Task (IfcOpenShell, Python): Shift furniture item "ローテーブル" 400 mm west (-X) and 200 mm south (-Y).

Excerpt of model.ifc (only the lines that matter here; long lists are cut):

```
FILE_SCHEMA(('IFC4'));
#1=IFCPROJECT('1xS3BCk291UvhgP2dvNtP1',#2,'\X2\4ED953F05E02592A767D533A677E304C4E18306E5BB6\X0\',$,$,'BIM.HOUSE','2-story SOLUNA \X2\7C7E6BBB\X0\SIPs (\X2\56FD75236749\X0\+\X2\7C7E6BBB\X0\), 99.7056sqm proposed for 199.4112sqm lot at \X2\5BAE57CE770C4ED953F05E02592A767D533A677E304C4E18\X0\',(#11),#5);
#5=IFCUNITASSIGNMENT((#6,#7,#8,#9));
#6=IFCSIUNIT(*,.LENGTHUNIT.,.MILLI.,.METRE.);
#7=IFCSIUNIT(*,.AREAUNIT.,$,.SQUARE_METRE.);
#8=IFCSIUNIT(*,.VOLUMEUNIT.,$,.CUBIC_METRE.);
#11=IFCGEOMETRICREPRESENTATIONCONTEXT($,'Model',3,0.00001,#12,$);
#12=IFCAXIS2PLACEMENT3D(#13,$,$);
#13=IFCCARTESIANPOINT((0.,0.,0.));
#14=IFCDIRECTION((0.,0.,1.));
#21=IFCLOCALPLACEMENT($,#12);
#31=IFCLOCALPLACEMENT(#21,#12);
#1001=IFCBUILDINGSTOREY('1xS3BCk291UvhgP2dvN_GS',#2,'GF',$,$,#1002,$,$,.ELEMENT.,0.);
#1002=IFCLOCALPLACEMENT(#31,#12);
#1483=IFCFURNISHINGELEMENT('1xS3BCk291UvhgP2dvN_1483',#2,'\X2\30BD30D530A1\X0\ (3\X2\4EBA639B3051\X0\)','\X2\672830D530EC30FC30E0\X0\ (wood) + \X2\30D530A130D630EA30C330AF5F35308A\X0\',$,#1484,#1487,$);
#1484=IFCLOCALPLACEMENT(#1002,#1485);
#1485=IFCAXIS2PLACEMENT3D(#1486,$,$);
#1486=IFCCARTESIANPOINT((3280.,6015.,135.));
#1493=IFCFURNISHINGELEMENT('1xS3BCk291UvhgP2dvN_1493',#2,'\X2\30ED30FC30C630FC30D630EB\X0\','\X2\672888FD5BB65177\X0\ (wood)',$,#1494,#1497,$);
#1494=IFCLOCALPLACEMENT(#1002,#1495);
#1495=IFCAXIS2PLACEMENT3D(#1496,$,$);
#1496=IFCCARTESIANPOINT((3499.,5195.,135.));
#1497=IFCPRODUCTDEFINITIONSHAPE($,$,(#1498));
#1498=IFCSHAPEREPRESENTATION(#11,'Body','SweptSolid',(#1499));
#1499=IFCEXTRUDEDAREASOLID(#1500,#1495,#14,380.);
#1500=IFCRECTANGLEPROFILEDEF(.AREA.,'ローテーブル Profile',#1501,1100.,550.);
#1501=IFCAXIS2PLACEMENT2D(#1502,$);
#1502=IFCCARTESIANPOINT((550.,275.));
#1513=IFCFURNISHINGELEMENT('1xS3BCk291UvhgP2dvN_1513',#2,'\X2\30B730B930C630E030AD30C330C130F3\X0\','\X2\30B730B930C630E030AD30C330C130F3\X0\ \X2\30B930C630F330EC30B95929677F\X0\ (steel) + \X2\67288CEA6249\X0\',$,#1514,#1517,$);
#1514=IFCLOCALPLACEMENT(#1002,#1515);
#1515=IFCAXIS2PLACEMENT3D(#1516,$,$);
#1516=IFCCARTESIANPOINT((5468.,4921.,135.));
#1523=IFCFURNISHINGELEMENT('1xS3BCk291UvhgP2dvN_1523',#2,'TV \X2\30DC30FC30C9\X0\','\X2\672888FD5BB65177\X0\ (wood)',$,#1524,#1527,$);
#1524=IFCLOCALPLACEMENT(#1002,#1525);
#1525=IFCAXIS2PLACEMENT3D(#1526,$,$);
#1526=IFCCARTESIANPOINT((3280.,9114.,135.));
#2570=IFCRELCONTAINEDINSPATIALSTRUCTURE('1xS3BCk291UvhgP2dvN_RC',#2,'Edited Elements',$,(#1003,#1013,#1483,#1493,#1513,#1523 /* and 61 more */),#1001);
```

```python
import ifcopenshell
import ifcopenshell.api.geometry
import ifcopenshell.util.placement
import ifcopenshell.util.unit

model = ifcopenshell.open("model.ifc")
unit_scale = ifcopenshell.util.unit.calculate_unit_scale(model)

item = model.by_guid("1xS3BCk291UvhgP2dvN_1493")
matrix = ifcopenshell.util.placement.get_local_placement(item.ObjectPlacement)
matrix[0, 3] -= 0.4 / unit_scale
matrix[1, 3] -= 0.2 / unit_scale
ifcopenshell.api.geometry.edit_object_placement(model, product=item, matrix=matrix, is_si=False)

print(ifcopenshell.util.placement.get_local_placement(item.ObjectPlacement).round(3) + 0.0)

model.write("model_edited.ifc")
```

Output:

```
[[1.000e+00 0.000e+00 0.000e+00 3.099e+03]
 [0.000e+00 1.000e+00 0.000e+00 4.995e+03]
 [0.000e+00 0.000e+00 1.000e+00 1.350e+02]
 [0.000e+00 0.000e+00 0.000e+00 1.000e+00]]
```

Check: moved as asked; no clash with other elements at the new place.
